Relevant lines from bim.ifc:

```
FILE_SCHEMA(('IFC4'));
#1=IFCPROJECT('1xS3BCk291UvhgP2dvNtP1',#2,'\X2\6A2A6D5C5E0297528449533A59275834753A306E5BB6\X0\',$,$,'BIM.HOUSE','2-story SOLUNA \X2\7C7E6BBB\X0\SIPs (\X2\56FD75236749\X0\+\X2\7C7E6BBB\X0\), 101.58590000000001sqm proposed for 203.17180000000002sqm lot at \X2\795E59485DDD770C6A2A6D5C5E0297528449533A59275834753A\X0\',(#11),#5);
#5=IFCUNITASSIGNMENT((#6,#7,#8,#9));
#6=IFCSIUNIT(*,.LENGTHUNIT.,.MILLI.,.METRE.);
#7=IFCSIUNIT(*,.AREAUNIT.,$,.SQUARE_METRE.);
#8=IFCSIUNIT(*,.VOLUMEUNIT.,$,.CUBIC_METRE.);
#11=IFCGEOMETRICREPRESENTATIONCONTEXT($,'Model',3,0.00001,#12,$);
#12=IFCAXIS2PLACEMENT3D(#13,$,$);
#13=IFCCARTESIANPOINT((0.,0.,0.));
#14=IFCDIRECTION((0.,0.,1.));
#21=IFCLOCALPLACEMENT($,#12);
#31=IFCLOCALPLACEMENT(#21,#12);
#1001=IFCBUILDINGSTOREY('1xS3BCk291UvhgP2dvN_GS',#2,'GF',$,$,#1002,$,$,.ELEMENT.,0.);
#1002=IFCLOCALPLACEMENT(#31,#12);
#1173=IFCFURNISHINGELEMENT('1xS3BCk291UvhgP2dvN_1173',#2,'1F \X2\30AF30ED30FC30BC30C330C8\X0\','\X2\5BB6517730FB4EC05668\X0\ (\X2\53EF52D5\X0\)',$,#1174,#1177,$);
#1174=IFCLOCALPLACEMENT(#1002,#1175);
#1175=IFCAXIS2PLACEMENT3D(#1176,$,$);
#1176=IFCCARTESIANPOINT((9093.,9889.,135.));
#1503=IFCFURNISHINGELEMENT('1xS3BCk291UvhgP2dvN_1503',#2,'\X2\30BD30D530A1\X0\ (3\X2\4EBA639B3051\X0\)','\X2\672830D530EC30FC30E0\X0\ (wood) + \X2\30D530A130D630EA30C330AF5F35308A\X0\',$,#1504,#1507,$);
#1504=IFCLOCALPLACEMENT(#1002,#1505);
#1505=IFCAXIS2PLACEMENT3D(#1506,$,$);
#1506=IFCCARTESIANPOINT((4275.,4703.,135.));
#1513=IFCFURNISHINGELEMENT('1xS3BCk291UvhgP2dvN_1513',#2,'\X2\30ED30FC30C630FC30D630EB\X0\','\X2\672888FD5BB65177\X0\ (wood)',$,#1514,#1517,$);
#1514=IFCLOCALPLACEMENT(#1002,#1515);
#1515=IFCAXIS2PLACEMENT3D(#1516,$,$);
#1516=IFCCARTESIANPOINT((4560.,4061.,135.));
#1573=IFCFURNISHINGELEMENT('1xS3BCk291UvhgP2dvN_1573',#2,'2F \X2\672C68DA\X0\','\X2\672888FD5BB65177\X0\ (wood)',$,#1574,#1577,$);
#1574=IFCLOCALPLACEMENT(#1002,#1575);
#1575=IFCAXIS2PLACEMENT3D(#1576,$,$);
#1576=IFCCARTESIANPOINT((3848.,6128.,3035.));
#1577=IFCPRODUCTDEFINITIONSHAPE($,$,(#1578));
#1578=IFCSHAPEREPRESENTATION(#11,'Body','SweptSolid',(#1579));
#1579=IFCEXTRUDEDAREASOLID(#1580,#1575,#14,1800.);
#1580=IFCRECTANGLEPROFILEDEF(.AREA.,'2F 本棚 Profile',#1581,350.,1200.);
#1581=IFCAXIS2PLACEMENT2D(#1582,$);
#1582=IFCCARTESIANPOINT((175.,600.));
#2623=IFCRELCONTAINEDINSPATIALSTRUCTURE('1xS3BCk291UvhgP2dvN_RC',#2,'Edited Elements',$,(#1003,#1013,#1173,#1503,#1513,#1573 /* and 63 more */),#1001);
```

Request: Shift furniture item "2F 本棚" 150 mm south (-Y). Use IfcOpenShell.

```python
import ifcopenshell
import ifcopenshell.api.geometry
import ifcopenshell.util.placement
import ifcopenshell.util.unit

model = ifcopenshell.open("bim.ifc")
unit_scale = ifcopenshell.util.unit.calculate_unit_scale(model)

item = model.by_guid("1xS3BCk291UvhgP2dvN_1573")
matrix = ifcopenshell.util.placement.get_local_placement(item.ObjectPlacement)
matrix[1, 3] -= 0.15 / unit_scale
ifcopenshell.api.geometry.edit_object_placement(model, product=item, matrix=matrix, is_si=False)

print(ifcopenshell.util.placement.get_local_placement(item.ObjectPlacement).round(3) + 0.0)

model.write("bim_rev.ifc")
```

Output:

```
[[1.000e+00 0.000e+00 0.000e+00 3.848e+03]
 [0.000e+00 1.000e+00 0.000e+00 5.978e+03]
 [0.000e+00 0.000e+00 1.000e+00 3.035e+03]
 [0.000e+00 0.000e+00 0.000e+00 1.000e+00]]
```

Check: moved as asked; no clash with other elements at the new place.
